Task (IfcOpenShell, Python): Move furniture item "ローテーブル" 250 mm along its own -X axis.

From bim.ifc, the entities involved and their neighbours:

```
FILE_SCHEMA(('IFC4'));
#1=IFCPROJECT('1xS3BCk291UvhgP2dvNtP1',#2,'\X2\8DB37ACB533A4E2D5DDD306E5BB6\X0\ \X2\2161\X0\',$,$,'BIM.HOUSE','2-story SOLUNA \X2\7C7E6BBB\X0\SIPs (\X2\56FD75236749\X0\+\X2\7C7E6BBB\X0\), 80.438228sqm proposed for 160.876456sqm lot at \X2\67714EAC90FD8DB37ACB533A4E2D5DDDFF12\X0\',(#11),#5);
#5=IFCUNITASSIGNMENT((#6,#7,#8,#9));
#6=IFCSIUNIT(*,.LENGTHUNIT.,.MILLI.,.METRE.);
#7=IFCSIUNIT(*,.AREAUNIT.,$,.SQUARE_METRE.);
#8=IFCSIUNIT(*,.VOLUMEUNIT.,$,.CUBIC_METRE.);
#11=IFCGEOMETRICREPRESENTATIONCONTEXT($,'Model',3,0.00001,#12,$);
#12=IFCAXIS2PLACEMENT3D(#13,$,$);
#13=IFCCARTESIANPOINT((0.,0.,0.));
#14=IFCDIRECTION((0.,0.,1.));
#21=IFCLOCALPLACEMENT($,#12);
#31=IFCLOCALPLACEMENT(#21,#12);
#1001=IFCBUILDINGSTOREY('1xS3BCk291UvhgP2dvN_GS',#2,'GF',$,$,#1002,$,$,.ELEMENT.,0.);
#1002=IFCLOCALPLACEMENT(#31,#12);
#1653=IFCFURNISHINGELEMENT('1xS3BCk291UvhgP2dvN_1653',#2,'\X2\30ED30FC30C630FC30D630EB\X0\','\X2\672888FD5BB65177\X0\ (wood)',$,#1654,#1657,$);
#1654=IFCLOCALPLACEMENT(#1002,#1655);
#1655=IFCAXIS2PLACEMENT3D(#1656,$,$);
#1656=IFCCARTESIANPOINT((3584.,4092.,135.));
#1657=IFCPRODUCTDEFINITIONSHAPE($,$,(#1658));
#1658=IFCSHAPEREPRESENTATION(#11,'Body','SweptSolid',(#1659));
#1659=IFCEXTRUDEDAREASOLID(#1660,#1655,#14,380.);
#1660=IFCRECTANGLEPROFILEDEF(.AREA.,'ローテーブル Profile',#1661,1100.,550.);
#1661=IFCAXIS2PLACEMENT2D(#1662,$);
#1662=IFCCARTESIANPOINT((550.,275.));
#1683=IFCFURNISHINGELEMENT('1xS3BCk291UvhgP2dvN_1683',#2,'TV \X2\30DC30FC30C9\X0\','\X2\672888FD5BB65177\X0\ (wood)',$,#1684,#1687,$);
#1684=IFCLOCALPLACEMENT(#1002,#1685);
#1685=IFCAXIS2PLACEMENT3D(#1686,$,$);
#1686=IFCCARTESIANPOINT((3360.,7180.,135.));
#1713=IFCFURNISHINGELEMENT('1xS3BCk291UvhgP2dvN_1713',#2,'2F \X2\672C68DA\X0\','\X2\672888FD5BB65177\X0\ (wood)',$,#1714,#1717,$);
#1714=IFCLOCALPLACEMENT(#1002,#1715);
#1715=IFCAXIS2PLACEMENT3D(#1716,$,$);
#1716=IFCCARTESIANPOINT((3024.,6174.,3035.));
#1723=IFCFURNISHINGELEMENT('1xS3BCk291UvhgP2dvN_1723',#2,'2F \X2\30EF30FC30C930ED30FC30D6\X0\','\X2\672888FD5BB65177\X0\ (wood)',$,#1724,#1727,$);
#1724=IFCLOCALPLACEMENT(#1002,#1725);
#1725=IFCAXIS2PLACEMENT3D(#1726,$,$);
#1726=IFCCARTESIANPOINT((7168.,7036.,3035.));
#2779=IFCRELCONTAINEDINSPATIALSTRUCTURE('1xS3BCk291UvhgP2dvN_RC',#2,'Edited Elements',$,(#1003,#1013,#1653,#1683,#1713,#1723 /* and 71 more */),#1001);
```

```python
import ifcopenshell
import ifcopenshell.api.geometry
import ifcopenshell.util.placement

model = ifcopenshell.open("bim.ifc")

item = model.by_guid("1xS3BCk291UvhgP2dvN_1653")
matrix = ifcopenshell.util.placement.get_local_placement(item.ObjectPlacement)
matrix[:3, 3] -= matrix[:3, 0] * 250.0
ifcopenshell.api.geometry.edit_object_placement(model, product=item, matrix=matrix, is_si=False)

print(ifcopenshell.util.placement.get_local_placement(item.ObjectPlacement).round(3) + 0.0)

model.write("bim_v2.ifc")
```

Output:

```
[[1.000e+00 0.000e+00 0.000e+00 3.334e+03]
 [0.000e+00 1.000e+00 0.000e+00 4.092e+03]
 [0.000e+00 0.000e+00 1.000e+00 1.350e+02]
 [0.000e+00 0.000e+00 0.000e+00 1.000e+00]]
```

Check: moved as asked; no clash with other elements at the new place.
